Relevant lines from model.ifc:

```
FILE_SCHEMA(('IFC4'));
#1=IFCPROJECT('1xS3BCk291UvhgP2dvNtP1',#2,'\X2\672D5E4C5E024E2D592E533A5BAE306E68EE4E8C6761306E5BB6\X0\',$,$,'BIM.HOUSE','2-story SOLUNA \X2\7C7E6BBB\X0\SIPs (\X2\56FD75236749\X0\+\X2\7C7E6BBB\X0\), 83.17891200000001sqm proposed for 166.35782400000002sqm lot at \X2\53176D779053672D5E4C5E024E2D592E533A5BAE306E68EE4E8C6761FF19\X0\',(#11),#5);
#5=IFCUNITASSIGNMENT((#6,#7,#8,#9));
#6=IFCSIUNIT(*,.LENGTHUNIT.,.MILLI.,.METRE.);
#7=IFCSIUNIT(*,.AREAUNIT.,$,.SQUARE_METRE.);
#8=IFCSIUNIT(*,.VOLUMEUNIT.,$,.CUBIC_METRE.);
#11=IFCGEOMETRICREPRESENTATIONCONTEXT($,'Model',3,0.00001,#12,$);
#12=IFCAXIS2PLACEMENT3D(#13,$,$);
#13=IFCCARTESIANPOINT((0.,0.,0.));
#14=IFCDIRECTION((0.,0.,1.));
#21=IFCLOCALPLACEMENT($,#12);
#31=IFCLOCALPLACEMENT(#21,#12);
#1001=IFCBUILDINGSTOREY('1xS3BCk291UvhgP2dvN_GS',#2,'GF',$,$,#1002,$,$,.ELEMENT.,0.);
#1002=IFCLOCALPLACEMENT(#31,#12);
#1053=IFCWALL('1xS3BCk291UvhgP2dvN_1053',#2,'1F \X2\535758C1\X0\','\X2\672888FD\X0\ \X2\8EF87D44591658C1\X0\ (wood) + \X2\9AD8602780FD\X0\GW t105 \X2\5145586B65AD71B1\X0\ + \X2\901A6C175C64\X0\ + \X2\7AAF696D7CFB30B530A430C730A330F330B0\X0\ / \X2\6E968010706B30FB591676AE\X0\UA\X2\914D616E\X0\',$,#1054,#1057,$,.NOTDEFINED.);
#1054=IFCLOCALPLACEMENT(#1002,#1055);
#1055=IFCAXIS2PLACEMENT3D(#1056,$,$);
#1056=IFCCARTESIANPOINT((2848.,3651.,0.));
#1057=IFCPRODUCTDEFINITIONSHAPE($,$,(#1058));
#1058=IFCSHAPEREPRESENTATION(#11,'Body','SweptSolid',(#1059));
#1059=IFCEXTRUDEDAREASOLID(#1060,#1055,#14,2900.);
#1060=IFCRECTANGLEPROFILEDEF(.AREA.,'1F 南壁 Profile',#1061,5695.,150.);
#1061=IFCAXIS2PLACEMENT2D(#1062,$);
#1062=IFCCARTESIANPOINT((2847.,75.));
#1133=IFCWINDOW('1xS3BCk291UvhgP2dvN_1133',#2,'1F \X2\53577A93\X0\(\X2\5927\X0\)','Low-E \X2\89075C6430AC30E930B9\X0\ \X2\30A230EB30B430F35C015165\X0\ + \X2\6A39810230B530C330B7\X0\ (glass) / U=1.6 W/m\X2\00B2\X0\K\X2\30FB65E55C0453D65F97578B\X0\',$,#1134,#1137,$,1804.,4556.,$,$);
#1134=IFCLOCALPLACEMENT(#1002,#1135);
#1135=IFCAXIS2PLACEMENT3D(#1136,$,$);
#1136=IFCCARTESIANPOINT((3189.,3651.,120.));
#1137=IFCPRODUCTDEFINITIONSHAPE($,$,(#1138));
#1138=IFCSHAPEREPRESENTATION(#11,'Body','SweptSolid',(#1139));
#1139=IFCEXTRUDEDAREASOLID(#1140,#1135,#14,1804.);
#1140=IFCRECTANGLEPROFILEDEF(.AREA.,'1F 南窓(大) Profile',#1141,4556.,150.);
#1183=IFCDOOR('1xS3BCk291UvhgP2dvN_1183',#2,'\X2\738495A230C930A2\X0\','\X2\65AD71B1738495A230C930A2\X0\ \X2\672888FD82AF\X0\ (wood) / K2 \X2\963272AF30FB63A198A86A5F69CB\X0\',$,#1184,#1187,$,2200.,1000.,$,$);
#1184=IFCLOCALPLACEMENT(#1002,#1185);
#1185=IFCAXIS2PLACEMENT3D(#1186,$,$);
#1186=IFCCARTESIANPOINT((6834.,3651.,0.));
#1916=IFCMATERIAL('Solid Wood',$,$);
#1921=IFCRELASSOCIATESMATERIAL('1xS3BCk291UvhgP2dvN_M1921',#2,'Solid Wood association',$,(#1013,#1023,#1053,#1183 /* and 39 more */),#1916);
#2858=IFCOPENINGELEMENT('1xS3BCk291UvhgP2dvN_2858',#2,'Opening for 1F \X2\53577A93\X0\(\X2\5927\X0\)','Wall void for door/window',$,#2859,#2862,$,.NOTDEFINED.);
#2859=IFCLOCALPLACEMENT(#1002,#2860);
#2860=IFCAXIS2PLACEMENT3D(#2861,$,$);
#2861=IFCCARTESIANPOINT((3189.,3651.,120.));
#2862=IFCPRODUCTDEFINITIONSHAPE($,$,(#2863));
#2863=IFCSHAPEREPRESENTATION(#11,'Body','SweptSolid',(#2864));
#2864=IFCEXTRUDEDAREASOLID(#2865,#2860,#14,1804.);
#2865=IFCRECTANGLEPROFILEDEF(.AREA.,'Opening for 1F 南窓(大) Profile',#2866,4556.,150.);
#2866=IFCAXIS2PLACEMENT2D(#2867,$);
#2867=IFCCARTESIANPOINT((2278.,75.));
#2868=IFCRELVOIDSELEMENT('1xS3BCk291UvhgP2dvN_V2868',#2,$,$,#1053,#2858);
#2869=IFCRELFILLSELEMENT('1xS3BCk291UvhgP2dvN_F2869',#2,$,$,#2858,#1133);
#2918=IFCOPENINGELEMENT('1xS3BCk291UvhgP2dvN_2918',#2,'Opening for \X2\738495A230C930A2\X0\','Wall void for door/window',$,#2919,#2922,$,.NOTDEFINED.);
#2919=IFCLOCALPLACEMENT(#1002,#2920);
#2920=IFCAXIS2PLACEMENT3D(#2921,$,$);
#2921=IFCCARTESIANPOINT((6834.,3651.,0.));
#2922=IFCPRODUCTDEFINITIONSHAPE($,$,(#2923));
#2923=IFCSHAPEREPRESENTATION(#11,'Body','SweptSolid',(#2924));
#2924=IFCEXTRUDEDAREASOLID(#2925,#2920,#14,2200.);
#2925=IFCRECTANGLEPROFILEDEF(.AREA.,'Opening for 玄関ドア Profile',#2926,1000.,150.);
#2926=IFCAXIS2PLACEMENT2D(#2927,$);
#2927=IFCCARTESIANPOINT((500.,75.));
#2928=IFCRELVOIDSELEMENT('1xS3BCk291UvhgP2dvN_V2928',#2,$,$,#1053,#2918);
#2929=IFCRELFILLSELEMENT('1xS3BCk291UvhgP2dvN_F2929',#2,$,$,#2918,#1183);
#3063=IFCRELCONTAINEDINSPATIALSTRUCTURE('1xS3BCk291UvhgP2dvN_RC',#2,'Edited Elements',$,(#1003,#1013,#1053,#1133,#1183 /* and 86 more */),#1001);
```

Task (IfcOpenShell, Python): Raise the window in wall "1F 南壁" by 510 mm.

```python
import numpy as np
import ifcopenshell
import ifcopenshell.api.geometry
import ifcopenshell.util.placement
import ifcopenshell.util.unit

model = ifcopenshell.open("model.ifc")
unit_scale = ifcopenshell.util.unit.calculate_unit_scale(model)

window = model.by_id(1133)
opening = window.FillsVoids[0].RelatingOpeningElement
dz = 510.0

shift = np.array([0.0, 0.0, dz])
# The window is not placed relative to its opening, so move both.
for product in (opening, window):
    matrix = ifcopenshell.util.placement.get_local_placement(product.ObjectPlacement)
    matrix[:3, 3] += shift
    ifcopenshell.api.geometry.edit_object_placement(model, product=product, matrix=matrix, is_si=False)

print(f"moved by {dz * unit_scale:+.3f} m")

model.write("model_updated.ifc")
```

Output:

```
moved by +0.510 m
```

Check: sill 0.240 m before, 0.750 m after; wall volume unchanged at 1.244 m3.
